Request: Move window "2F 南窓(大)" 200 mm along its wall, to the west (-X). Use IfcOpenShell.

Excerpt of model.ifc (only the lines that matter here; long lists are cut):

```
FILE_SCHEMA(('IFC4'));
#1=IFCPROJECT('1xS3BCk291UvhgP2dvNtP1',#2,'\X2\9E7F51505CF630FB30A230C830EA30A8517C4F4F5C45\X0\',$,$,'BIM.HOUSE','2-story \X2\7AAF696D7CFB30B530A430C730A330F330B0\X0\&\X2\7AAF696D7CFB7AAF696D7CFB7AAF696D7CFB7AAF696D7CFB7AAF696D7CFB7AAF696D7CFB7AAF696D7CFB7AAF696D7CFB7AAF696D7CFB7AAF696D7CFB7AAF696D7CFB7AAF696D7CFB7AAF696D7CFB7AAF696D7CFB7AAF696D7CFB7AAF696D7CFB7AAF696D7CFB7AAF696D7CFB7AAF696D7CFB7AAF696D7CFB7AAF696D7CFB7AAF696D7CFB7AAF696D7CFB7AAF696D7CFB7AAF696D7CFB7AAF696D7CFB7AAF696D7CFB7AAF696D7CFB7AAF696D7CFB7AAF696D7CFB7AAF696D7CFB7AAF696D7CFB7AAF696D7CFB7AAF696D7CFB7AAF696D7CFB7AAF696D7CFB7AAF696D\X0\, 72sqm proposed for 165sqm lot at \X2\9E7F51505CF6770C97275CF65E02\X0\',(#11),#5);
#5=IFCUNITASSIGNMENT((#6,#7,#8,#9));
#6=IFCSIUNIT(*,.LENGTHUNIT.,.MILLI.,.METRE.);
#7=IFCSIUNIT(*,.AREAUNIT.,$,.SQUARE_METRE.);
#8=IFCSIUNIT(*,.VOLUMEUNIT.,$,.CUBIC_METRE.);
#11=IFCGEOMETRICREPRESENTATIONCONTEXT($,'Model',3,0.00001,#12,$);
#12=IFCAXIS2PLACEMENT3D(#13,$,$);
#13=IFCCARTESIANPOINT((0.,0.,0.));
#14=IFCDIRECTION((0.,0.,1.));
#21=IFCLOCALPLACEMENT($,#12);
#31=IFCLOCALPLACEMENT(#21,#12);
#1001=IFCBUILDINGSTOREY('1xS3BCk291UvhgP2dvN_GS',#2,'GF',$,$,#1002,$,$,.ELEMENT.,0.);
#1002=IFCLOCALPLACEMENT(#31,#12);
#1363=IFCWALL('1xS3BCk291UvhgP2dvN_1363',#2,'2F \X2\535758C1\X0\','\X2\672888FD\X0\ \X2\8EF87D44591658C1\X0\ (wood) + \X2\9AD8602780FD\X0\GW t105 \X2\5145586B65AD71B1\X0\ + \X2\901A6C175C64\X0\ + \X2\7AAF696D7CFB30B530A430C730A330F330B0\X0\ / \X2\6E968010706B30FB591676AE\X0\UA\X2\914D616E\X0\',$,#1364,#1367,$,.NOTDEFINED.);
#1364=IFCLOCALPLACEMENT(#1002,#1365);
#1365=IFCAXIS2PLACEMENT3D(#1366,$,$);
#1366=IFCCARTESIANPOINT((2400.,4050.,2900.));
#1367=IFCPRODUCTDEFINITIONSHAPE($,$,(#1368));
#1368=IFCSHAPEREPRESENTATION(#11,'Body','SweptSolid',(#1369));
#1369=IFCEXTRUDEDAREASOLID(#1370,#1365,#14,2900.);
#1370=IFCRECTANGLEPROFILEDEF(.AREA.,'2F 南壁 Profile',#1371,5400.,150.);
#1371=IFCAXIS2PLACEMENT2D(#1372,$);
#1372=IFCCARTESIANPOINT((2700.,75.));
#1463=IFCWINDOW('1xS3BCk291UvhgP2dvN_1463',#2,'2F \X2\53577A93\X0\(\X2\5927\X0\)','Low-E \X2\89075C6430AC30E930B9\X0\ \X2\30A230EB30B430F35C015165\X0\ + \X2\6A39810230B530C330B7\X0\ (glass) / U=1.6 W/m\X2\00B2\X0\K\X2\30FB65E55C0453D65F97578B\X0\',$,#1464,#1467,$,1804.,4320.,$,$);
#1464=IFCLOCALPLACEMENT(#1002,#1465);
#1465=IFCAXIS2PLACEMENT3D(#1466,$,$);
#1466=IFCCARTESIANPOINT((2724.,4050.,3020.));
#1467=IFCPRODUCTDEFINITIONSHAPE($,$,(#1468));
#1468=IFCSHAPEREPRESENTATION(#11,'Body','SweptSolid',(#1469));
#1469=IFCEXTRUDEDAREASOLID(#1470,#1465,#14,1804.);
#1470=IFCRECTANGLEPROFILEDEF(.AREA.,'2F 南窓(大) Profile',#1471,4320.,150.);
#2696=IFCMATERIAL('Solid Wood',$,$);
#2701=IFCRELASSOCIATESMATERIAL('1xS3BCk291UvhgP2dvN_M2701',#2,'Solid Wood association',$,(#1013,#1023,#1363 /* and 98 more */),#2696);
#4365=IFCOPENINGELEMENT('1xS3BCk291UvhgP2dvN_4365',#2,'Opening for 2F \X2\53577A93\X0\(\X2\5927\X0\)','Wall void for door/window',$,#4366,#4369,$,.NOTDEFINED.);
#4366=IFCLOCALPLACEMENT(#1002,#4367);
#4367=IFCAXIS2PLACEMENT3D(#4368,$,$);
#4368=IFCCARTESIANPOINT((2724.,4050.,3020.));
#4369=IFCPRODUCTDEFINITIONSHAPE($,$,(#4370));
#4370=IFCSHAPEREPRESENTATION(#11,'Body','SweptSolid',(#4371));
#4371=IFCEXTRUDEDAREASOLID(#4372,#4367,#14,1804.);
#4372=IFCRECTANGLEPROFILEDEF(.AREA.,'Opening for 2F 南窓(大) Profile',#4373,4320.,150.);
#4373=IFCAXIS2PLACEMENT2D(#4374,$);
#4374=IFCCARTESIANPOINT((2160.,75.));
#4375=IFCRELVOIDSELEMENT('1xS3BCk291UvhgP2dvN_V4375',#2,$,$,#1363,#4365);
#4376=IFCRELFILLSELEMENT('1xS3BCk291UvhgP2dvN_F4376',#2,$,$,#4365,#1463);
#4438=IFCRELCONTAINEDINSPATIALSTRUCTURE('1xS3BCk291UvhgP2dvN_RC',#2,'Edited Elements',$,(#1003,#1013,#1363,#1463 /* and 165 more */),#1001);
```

```python
import ifcopenshell
import ifcopenshell.api.geometry
import ifcopenshell.util.placement

model = ifcopenshell.open("model.ifc")

window = model.by_guid("1xS3BCk291UvhgP2dvN_1463")
opening = window.FillsVoids[0].RelatingOpeningElement
wall = opening.VoidsElements[0].RelatingBuildingElement

wall_matrix = ifcopenshell.util.placement.get_local_placement(wall.ObjectPlacement)
shift = wall_matrix[:3, 0] * -200.0
before = ifcopenshell.util.placement.get_local_placement(window.ObjectPlacement)[:3, 3].copy()

# The window is not placed relative to its opening, so move both.
for product in (opening, window):
    matrix = ifcopenshell.util.placement.get_local_placement(product.ObjectPlacement)
    matrix[:3, 3] += shift
    ifcopenshell.api.geometry.edit_object_placement(model, product=product, matrix=matrix, is_si=False)

after = ifcopenshell.util.placement.get_local_placement(window.ObjectPlacement)[:3, 3]
print("window moved by", (after - before).round(3) + 0.0)

model.write("model-out.ifc")
```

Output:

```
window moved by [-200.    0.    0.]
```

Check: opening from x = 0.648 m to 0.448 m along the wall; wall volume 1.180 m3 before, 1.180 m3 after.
